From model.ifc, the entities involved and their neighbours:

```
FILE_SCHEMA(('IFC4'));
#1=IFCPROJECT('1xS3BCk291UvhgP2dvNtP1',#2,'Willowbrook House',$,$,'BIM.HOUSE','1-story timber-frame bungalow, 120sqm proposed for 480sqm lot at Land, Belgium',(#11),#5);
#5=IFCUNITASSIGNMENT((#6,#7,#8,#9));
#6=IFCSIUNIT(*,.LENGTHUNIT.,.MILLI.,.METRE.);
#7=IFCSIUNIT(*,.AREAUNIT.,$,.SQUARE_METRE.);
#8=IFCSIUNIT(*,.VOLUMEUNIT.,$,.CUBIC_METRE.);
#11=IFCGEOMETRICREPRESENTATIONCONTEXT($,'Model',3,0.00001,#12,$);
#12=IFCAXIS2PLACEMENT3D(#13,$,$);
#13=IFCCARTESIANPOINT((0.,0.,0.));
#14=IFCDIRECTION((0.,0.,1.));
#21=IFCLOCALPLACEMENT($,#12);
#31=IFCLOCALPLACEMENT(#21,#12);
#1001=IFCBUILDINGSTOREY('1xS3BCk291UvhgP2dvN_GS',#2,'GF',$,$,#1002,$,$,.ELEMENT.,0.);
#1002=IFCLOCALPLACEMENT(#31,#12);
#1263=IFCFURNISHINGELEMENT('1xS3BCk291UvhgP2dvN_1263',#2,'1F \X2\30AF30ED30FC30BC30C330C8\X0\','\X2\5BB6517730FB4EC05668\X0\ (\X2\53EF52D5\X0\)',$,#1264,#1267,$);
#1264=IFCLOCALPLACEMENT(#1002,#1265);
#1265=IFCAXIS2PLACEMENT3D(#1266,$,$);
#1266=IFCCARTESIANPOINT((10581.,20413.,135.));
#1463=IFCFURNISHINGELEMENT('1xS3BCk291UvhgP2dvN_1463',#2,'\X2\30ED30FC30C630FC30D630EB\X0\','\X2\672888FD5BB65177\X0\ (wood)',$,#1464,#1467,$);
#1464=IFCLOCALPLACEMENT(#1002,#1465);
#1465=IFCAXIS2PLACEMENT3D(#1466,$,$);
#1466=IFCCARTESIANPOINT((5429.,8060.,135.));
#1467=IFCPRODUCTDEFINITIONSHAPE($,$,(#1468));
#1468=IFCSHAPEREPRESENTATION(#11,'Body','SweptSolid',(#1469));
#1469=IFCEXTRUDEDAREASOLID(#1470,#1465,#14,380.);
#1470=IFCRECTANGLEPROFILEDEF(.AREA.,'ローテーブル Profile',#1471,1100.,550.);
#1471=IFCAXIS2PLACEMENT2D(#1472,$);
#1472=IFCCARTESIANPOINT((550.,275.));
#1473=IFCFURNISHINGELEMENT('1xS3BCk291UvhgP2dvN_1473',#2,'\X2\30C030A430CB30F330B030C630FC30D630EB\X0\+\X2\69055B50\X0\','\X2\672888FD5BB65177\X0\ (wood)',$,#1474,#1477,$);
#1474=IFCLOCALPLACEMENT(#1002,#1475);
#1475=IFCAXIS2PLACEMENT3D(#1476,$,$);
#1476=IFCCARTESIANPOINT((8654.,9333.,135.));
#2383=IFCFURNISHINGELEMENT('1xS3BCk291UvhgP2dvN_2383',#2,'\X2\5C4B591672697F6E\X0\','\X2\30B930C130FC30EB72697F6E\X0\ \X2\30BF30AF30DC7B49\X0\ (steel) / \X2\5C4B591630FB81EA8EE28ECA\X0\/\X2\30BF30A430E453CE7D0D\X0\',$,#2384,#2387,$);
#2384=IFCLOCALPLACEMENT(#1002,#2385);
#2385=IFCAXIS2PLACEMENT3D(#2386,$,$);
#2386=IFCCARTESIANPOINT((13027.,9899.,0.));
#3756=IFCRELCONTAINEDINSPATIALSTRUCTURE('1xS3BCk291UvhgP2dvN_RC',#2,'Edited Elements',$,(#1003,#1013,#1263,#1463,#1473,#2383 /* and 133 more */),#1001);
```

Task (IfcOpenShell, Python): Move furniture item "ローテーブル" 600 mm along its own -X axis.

```python
import ifcopenshell
import ifcopenshell.api.geometry
import ifcopenshell.util.placement

model = ifcopenshell.open("model.ifc")

item = model.by_guid("1xS3BCk291UvhgP2dvN_1463")
matrix = ifcopenshell.util.placement.get_local_placement(item.ObjectPlacement)
matrix[:3, 3] -= matrix[:3, 0] * 600.0
ifcopenshell.api.geometry.edit_object_placement(model, product=item, matrix=matrix, is_si=False)

print(ifcopenshell.util.placement.get_local_placement(item.ObjectPlacement).round(3) + 0.0)

model.write("model_updated.ifc")
```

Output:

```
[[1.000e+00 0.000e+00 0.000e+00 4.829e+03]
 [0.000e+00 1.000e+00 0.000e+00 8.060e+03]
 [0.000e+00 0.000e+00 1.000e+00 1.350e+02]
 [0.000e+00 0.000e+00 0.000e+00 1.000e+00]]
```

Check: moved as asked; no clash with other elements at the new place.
